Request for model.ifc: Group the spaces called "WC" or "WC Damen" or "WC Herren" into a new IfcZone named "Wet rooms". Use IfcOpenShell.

First a look at what the model holds.

```python
import ifcopenshell

model = ifcopenshell.open("model.ifc")
print(model.schema)
seen = {}
for space in model.by_type("IfcSpace"):
    seen[space.LongName] = seen.get(space.LongName, 0) + 1
for name, count in sorted(seen.items(), key=str):
    print(count, "x", name)
print("zones:", [z.Name for z in model.by_type("IfcZone")][:20])
```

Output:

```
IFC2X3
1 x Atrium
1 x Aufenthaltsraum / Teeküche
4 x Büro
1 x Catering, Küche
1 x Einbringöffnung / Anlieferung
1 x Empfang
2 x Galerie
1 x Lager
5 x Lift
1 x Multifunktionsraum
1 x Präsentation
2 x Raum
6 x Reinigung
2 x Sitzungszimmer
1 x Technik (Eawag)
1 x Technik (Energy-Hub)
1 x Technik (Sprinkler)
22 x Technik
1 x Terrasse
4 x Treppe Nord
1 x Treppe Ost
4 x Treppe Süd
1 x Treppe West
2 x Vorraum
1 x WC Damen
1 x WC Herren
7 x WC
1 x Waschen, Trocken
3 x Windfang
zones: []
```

```python
import ifcopenshell
import ifcopenshell.api.group
import ifcopenshell.api.root

model = ifcopenshell.open("model.ifc")

names = {"WC", "WC Damen", "WC Herren"}
spaces = [s for s in model.by_type("IfcSpace") if s.LongName in names]

zone = ifcopenshell.api.root.create_entity(model, ifc_class="IfcZone", name="Wet rooms")
ifcopenshell.api.group.assign_group(model, products=spaces, group=zone)
print(len(spaces), "spaces in", zone.Name)

model.write("model_updated.ifc")
```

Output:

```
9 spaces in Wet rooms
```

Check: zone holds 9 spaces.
